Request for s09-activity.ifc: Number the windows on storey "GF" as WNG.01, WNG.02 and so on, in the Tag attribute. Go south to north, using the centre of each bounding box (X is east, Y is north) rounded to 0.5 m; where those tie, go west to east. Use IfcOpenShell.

First a look at what the model holds.

```python
import ifcopenshell
import ifcopenshell.util.element
import ifcopenshell.util.placement

model = ifcopenshell.open("s09-activity.ifc")
print(model.schema)
storey = next(s for s in model.by_type("IfcBuildingStorey") if s.Name == "GF")
windows = [e for e in ifcopenshell.util.element.get_decomposition(storey) if e.is_a("IfcWindow")]
for e in sorted(windows, key=lambda e: e.id()):
    origin = ifcopenshell.util.placement.get_local_placement(e.ObjectPlacement)[:3, 3]
    print(e.id(), e.Tag, e.Name, origin.round(2) + 0.0, sep=" | ")
```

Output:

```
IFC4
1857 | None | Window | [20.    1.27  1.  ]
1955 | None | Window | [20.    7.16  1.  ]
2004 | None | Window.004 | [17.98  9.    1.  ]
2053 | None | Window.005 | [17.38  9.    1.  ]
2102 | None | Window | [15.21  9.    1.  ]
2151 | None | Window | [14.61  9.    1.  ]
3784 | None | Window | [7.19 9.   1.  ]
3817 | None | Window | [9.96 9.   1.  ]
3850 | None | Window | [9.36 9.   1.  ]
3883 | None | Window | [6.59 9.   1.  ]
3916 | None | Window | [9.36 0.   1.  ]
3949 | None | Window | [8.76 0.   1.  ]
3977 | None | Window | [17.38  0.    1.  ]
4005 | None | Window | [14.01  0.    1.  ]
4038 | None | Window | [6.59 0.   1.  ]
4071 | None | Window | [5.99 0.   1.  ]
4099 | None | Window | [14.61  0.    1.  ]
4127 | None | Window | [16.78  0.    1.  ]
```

```python
import ifcopenshell
import ifcopenshell.geom
import ifcopenshell.util.element
import ifcopenshell.util.shape

model = ifcopenshell.open("s09-activity.ifc")
settings = ifcopenshell.geom.settings()
settings.set("use-world-coords", True)


def centre(element):
    shape = ifcopenshell.geom.create_shape(settings, element)
    return ifcopenshell.util.shape.get_bbox_centroid(shape.geometry)


storey = next(s for s in model.by_type("IfcBuildingStorey") if s.Name == "GF")
windows = [e for e in ifcopenshell.util.element.get_decomposition(storey) if e.is_a("IfcWindow")]

# Insertion points can sit at a corner or the storey origin, so sort by the geometry (in metres).
centres = {e: centre(e) for e in windows}
windows.sort(key=lambda e: (round(centres[e][1] / 0.5), centres[e][0]))

for i, e in enumerate(windows, start=1):
    number = f"WNG.{i:02d}"
    e.Tag = number
    print(e.id(), number)

model.write("s09-activity_updated.ifc")
```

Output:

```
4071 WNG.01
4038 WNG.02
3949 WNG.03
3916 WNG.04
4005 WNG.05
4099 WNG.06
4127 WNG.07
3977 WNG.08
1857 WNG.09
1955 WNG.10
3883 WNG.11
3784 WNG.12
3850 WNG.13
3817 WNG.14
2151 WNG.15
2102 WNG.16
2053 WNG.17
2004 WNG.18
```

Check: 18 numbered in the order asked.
